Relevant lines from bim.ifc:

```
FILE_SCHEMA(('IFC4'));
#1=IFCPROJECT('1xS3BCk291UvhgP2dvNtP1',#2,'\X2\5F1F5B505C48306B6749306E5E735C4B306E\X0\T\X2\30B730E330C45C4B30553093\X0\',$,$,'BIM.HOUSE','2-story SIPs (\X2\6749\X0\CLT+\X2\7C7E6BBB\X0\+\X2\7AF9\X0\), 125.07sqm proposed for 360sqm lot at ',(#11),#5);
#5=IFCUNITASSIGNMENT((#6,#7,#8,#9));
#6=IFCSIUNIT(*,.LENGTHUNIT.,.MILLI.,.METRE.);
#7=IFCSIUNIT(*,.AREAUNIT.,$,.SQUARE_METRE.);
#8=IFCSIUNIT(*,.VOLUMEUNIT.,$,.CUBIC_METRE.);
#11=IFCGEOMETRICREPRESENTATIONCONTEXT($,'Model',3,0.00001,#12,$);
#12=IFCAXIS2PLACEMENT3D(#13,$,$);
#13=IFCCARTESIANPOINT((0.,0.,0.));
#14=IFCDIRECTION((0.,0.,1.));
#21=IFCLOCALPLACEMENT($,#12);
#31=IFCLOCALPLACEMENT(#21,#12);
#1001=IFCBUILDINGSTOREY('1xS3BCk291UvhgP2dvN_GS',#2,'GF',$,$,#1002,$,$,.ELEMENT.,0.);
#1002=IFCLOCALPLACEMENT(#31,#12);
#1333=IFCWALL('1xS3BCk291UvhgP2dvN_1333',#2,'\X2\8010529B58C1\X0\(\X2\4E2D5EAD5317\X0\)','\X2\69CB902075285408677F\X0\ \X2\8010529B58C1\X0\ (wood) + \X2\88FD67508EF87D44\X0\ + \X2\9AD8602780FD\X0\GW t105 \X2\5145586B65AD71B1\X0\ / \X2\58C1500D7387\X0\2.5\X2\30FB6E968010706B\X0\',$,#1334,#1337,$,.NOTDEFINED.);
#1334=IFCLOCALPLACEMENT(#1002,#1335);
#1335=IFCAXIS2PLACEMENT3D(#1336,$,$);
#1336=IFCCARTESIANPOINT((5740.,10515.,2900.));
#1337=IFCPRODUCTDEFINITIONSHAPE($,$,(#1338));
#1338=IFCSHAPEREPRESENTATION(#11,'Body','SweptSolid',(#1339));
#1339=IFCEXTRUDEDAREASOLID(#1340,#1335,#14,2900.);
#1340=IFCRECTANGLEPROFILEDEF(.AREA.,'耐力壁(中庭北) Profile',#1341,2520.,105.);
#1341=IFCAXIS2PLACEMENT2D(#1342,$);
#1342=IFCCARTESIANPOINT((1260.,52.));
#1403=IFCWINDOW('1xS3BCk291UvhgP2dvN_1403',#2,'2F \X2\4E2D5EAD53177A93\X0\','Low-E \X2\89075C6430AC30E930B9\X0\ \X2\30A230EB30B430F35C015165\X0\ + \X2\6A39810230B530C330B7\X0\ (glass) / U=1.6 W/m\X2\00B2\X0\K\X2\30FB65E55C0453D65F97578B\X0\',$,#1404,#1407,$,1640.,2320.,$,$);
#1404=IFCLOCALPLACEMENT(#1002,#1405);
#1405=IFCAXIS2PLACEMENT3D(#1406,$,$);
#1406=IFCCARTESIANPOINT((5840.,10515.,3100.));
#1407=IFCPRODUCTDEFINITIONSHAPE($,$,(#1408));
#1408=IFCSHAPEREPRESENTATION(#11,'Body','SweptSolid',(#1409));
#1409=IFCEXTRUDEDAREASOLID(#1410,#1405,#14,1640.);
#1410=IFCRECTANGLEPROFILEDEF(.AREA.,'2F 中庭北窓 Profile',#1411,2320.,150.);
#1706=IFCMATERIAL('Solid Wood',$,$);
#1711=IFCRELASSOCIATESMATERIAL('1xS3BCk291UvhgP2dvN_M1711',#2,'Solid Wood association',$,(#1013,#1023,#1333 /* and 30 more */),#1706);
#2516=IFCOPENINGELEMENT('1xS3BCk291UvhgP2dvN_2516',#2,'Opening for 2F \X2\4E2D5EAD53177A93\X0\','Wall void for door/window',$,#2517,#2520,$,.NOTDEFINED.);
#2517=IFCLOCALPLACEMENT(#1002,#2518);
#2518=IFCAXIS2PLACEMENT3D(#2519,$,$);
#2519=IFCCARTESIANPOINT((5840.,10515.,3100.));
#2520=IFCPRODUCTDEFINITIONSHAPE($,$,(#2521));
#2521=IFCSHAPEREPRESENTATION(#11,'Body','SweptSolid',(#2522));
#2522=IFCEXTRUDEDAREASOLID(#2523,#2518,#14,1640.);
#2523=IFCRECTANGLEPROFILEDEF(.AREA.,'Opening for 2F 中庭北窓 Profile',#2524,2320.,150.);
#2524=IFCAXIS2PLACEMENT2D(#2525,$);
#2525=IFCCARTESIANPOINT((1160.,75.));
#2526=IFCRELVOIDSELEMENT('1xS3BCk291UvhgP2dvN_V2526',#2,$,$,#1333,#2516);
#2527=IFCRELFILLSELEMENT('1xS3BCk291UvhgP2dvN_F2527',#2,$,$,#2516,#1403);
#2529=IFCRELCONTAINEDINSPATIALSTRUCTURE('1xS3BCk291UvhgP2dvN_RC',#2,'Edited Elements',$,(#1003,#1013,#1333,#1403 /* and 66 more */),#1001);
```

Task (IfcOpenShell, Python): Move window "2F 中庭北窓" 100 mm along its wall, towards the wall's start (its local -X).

```python
import ifcopenshell
import ifcopenshell.api.geometry
import ifcopenshell.util.placement
import ifcopenshell.util.unit

model = ifcopenshell.open("bim.ifc")
unit_scale = ifcopenshell.util.unit.calculate_unit_scale(model)

window = model.by_id(1403)
opening = window.FillsVoids[0].RelatingOpeningElement
wall = opening.VoidsElements[0].RelatingBuildingElement

wall_matrix = ifcopenshell.util.placement.get_local_placement(wall.ObjectPlacement)
shift = wall_matrix[:3, 0] * -0.1 / unit_scale
before = ifcopenshell.util.placement.get_local_placement(window.ObjectPlacement)[:3, 3].copy()

# The window is not placed relative to its opening, so move both.
for product in (opening, window):
    matrix = ifcopenshell.util.placement.get_local_placement(product.ObjectPlacement)
    matrix[:3, 3] += shift
    ifcopenshell.api.geometry.edit_object_placement(model, product=product, matrix=matrix, is_si=False)

after = ifcopenshell.util.placement.get_local_placement(window.ObjectPlacement)[:3, 3]
print("window moved by", (after - before).round(3) + 0.0)

model.write("bim_rev.ifc")
```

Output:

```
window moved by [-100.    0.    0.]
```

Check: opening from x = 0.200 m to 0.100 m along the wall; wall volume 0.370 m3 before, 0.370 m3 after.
